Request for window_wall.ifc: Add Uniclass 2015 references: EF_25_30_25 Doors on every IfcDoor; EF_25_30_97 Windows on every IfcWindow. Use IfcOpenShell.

First a look at what the model holds.

```python
import ifcopenshell

model = ifcopenshell.open("window_wall.ifc")
print(model.schema)
print("classifications:", [c.Name for c in model.by_type("IfcClassification")])
for ifc_class in ("IfcDoor", "IfcRoof", "IfcStair", "IfcWall", "IfcWindow"):
    print(ifc_class, len(model.by_type(ifc_class)))
```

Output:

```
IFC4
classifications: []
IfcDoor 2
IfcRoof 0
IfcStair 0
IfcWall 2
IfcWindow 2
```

```python
import ifcopenshell
import ifcopenshell.api.classification

model = ifcopenshell.open("window_wall.ifc")

system = ifcopenshell.api.classification.add_classification(model, classification="Uniclass 2015")

codes = {
    "IfcDoor": ("EF_25_30_25", "Doors"),
    "IfcWindow": ("EF_25_30_97", "Windows"),
}
for ifc_class, (code, name) in codes.items():
    products = model.by_type(ifc_class)
    ifcopenshell.api.classification.add_reference(
        model, products=products, classification=system, identification=code, name=name
    )
    print(code, len(products))

model.write("window_wall_updated.ifc")
```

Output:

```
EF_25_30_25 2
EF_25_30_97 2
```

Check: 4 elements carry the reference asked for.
